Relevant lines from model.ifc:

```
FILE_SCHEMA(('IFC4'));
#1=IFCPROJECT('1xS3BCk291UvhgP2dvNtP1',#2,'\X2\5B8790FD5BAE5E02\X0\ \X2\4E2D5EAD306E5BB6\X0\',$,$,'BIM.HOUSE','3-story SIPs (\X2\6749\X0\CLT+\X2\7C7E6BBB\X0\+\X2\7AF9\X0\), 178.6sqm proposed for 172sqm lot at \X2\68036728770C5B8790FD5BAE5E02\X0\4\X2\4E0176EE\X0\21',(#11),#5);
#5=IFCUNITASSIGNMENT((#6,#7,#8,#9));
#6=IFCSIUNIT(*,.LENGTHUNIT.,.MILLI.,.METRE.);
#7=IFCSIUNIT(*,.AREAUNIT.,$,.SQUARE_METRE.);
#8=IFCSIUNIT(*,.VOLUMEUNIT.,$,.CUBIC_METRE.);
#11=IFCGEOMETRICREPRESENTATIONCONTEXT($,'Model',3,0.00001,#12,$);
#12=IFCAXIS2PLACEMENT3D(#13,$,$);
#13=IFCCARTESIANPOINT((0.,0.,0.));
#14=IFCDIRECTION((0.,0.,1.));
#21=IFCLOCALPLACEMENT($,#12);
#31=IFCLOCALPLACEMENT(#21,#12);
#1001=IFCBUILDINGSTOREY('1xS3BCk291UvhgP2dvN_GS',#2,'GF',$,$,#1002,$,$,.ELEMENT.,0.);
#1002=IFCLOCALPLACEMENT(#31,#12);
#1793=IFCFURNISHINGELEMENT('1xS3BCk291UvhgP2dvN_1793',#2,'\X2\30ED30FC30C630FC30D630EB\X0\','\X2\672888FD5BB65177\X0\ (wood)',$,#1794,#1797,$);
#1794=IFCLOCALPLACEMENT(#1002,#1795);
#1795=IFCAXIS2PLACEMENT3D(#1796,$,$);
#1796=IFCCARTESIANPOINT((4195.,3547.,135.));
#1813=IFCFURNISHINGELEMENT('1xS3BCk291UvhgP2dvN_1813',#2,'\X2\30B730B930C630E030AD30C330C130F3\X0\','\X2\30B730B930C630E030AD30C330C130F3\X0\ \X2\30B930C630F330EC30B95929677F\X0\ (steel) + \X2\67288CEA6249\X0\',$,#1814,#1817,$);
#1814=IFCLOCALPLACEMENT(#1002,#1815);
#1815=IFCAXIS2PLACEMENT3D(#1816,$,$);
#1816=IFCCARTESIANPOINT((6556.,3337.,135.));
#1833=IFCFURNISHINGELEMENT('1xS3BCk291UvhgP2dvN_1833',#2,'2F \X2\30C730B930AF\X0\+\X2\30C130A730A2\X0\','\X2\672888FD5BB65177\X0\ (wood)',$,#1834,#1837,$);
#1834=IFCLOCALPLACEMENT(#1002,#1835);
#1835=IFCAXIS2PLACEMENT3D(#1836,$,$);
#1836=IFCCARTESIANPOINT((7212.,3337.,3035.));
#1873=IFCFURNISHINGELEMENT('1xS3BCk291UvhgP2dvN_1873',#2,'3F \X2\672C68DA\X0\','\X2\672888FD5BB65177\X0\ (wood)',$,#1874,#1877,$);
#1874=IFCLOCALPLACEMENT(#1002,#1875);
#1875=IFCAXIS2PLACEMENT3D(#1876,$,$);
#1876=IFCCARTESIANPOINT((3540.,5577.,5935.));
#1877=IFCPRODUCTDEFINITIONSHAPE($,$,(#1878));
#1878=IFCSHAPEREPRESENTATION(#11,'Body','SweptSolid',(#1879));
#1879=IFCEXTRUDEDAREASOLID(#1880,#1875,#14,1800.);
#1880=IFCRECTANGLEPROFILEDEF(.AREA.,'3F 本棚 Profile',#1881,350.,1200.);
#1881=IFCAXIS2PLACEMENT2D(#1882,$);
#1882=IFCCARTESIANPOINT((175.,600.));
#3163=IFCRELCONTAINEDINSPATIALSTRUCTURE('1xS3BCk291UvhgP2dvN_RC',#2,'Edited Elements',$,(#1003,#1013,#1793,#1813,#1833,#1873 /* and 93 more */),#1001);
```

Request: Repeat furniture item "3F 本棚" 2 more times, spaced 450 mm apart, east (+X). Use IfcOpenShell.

```python
import numpy as np
import ifcopenshell
import ifcopenshell.api.geometry
import ifcopenshell.api.root
import ifcopenshell.util.element
import ifcopenshell.util.placement
import ifcopenshell.util.unit

model = ifcopenshell.open("model.ifc")
unit_scale = ifcopenshell.util.unit.calculate_unit_scale(model)


def reuse_history(source, copy):
    """copy_class also copies each property set's owner history, people and application; keep the originals."""
    for rel in copy.IsDefinedBy:
        if rel.is_a("IfcRelDefinesByProperties") and (history := rel.RelatingPropertyDefinition.OwnerHistory):
            rel.RelatingPropertyDefinition.OwnerHistory = source.OwnerHistory
            ifcopenshell.util.element.remove_deep2(model, history)


source = model.by_guid("1xS3BCk291UvhgP2dvN_1873")
base = ifcopenshell.util.placement.get_local_placement(source.ObjectPlacement)
step = np.array([1.0, 0.0, 0.0]) * 0.45 / unit_scale

for i in range(1, 3):
    copy = ifcopenshell.api.root.copy_class(model, product=source)
    copy.Representation = ifcopenshell.util.element.copy_deep(
        model, source.Representation, exclude=["IfcGeometricRepresentationContext", "IfcRepresentationMap"]
    )
    reuse_history(source, copy)
    matrix = base.copy()
    matrix[:3, 3] += i * step
    print("added at", matrix[:3, 3].round(3) + 0.0)
    ifcopenshell.api.geometry.edit_object_placement(model, product=copy, matrix=matrix, is_si=False)

model.write("model_rev.ifc")
```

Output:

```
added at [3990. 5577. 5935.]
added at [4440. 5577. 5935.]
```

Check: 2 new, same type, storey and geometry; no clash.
